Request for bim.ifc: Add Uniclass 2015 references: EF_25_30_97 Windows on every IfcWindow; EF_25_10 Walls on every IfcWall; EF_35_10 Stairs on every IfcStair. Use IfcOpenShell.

First a look at what the model holds.

```python
import ifcopenshell

model = ifcopenshell.open("bim.ifc")
print(model.schema)
print("classifications:", [c.Name for c in model.by_type("IfcClassification")])
for ifc_class in ("IfcDoor", "IfcRoof", "IfcStair", "IfcWall", "IfcWindow"):
    print(ifc_class, len(model.by_type(ifc_class)))
```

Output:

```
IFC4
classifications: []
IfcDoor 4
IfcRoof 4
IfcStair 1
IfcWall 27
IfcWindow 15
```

```python
import ifcopenshell
import ifcopenshell.api.classification

model = ifcopenshell.open("bim.ifc")

system = ifcopenshell.api.classification.add_classification(model, classification="Uniclass 2015")

codes = {
    "IfcWindow": ("EF_25_30_97", "Windows"),
    "IfcWall": ("EF_25_10", "Walls"),
    "IfcStair": ("EF_35_10", "Stairs"),
}
for ifc_class, (code, name) in codes.items():
    products = model.by_type(ifc_class)
    ifcopenshell.api.classification.add_reference(
        model, products=products, classification=system, identification=code, name=name
    )
    print(code, len(products))

model.write("bim_v2.ifc")
```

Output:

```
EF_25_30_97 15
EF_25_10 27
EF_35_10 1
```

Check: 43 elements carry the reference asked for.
